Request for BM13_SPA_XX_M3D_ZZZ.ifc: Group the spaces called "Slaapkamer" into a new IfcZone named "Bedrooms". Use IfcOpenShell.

First a look at what the model holds.

```python
import ifcopenshell

model = ifcopenshell.open("BM13_SPA_XX_M3D_ZZZ.ifc")
print(model.schema)
seen = {}
for space in model.by_type("IfcSpace"):
    seen[space.LongName] = seen.get(space.LongName, 0) + 1
for name, count in sorted(seen.items(), key=str):
    print(count, "x", name)
print("zones:", [z.Name for z in model.by_type("IfcZone")][:20])
```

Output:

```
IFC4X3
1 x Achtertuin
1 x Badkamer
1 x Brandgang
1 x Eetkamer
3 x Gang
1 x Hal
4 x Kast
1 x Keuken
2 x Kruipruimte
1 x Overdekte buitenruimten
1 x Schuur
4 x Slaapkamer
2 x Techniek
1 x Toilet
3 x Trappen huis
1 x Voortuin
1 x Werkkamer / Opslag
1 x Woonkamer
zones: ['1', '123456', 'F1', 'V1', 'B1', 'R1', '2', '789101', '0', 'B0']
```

```python
import ifcopenshell
import ifcopenshell.api.group
import ifcopenshell.api.root

model = ifcopenshell.open("BM13_SPA_XX_M3D_ZZZ.ifc")

names = {"Slaapkamer"}
spaces = [s for s in model.by_type("IfcSpace") if s.LongName in names]

zone = ifcopenshell.api.root.create_entity(model, ifc_class="IfcZone", name="Bedrooms")
ifcopenshell.api.group.assign_group(model, products=spaces, group=zone)
print(len(spaces), "spaces in", zone.Name)

model.write("BM13_SPA_XX_M3D_ZZZ_v2.ifc")
```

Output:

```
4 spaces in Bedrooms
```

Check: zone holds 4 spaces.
